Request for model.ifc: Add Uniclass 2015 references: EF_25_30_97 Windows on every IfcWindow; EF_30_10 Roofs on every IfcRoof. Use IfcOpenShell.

First a look at what the model holds.

```python
import ifcopenshell

model = ifcopenshell.open("model.ifc")
print(model.schema)
print("classifications:", [c.Name for c in model.by_type("IfcClassification")])
for ifc_class in ("IfcDoor", "IfcRoof", "IfcStair", "IfcWall", "IfcWindow"):
    print(ifc_class, len(model.by_type(ifc_class)))
```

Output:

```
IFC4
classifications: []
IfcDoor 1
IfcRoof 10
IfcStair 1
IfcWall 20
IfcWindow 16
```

```python
import ifcopenshell
import ifcopenshell.api.classification

model = ifcopenshell.open("model.ifc")

system = ifcopenshell.api.classification.add_classification(model, classification="Uniclass 2015")

codes = {
    "IfcWindow": ("EF_25_30_97", "Windows"),
    "IfcRoof": ("EF_30_10", "Roofs"),
}
for ifc_class, (code, name) in codes.items():
    products = model.by_type(ifc_class)
    ifcopenshell.api.classification.add_reference(
        model, products=products, classification=system, identification=code, name=name
    )
    print(code, len(products))

model.write("model_edited.ifc")
```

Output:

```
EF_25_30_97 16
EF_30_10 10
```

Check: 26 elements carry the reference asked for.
